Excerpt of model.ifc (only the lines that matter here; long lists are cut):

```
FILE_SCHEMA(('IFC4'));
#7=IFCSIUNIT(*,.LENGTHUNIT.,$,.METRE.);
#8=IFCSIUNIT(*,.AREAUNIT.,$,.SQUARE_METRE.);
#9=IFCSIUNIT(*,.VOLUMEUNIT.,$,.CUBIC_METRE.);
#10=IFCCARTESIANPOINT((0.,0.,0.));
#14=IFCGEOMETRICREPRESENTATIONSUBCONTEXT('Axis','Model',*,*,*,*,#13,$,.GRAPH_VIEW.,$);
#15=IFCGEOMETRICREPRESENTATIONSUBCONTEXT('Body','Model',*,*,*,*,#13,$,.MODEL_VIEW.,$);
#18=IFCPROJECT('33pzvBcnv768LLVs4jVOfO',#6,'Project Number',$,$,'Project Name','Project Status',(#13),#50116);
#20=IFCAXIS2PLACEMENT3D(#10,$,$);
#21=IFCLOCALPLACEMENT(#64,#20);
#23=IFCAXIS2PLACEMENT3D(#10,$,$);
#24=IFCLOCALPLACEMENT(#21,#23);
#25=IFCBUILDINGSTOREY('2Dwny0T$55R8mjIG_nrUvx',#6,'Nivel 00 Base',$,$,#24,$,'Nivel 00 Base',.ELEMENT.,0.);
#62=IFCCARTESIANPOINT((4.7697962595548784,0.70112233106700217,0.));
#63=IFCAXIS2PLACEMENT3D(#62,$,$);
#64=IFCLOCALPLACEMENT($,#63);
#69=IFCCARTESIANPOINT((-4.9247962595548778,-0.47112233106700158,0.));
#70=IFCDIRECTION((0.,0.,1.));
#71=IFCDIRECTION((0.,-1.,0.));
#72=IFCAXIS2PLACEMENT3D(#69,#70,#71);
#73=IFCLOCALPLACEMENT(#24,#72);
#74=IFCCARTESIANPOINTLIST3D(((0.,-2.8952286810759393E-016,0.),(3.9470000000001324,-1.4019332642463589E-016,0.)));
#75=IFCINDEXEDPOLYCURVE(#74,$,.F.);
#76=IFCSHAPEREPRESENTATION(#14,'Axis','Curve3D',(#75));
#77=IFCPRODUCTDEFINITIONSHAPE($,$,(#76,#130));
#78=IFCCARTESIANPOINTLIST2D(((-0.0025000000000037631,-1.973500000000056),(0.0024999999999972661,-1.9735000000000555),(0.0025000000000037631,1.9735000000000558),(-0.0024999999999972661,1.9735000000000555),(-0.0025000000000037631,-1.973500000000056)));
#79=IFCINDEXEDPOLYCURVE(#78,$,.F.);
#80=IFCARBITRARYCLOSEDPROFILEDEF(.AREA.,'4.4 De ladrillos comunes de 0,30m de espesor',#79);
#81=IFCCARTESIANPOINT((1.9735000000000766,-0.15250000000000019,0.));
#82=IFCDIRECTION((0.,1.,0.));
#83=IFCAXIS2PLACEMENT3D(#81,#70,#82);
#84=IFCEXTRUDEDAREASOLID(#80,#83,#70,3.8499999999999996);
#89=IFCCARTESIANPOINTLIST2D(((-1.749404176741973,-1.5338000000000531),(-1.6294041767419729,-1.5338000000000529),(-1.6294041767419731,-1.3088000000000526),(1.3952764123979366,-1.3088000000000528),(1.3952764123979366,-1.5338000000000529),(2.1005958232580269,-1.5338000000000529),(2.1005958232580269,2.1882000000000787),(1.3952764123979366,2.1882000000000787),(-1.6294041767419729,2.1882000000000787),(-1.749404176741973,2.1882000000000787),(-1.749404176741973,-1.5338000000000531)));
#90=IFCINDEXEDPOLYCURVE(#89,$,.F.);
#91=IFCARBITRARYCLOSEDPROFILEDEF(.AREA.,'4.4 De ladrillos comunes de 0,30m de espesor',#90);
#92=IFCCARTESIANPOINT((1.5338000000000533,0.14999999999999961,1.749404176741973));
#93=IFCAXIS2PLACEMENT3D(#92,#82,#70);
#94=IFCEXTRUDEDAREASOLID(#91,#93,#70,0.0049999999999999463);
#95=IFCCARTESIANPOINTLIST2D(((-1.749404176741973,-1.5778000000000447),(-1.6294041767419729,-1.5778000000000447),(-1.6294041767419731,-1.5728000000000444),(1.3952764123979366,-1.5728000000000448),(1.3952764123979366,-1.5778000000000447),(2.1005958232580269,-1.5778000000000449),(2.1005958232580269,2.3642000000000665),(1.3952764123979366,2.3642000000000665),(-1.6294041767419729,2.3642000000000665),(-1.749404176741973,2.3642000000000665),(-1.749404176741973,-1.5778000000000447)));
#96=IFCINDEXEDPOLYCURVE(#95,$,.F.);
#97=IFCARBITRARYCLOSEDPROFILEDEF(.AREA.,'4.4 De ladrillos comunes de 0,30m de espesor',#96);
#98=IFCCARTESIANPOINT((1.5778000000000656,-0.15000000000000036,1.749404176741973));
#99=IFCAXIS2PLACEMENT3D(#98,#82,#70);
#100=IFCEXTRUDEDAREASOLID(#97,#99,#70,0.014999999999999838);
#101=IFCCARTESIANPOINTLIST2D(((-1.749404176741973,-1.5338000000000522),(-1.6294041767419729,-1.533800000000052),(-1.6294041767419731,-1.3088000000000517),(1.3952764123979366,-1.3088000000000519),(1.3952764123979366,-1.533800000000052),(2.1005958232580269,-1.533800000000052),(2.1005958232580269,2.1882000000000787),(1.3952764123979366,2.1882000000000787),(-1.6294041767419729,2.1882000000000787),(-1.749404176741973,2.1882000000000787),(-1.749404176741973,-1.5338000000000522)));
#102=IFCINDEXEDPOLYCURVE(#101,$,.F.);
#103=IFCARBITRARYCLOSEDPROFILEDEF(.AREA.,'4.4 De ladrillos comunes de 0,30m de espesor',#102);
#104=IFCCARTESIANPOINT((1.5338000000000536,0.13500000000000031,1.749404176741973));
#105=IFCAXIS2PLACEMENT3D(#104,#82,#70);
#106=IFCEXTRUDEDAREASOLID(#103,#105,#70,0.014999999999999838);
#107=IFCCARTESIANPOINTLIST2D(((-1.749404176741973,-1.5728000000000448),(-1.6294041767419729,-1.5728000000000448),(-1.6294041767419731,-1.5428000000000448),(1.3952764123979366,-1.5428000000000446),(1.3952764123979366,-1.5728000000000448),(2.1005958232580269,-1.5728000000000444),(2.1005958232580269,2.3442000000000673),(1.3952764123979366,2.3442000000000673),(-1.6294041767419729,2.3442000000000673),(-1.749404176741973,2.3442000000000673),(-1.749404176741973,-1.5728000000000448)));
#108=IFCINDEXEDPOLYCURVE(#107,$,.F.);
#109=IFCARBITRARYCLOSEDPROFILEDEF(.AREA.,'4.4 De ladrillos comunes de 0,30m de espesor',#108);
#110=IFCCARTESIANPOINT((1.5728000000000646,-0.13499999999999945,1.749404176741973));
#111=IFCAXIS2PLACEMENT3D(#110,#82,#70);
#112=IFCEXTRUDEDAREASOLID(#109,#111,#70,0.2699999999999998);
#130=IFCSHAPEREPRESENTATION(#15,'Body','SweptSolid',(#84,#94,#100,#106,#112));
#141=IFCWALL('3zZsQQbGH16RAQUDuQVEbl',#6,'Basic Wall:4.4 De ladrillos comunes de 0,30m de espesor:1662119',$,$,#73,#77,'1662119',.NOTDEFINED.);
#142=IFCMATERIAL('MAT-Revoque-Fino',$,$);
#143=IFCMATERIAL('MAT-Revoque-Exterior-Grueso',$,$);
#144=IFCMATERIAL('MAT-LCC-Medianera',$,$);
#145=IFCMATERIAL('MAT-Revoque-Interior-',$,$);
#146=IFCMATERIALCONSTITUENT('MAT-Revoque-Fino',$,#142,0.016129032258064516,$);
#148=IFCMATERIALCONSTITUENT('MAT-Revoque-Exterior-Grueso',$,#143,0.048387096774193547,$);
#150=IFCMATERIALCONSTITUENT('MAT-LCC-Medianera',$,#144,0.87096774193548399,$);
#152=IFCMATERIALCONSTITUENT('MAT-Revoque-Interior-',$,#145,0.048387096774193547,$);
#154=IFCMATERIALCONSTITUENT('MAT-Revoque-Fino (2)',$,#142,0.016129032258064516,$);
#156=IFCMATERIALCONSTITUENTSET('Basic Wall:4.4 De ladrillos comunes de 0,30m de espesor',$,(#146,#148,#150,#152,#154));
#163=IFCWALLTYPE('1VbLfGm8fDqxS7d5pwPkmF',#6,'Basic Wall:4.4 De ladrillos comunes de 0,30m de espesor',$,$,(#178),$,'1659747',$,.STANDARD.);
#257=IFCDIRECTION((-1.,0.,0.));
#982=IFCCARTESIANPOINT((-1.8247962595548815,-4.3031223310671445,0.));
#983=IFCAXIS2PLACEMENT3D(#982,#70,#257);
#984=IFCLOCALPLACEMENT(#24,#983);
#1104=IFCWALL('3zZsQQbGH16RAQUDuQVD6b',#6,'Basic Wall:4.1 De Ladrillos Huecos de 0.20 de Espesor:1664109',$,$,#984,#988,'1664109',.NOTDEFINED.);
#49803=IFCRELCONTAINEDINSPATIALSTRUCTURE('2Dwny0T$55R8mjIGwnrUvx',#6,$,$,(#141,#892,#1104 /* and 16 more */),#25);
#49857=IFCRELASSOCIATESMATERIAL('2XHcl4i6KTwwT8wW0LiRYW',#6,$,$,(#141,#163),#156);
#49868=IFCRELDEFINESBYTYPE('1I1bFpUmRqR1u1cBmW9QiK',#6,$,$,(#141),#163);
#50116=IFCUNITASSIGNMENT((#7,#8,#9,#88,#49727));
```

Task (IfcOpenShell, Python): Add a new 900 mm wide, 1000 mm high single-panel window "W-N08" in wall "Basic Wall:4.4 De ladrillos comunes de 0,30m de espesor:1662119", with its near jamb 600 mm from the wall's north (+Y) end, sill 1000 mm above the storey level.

```python
import numpy as np
import ifcopenshell
import ifcopenshell.api.feature
import ifcopenshell.api.geometry
import ifcopenshell.api.root
import ifcopenshell.api.spatial
import ifcopenshell.geom
import ifcopenshell.util.element
import ifcopenshell.util.placement
import ifcopenshell.util.representation
import ifcopenshell.util.shape
import ifcopenshell.util.unit

model = ifcopenshell.open("model.ifc")
unit_scale = ifcopenshell.util.unit.calculate_unit_scale(model)
settings = ifcopenshell.geom.settings()


def volume(element):
    """Net volume in cubic metres, openings subtracted."""
    shape = ifcopenshell.geom.create_shape(settings, element)
    return ifcopenshell.util.shape.get_volume(shape.geometry)


wall = model.by_guid("3zZsQQbGH16RAQUDuQVEbl")
storey = ifcopenshell.util.element.get_container(wall, ifc_class="IfcBuildingStorey")
context = ifcopenshell.util.representation.get_context(model, "Model", "Body", "MODEL_VIEW")
before = volume(wall)

width, height, from_end, sill = 0.9, 1, 0.6, 1  # metres

# The wall runs along its own X axis, and the end named is its -X end.
wall_shape = ifcopenshell.geom.create_shape(settings, wall)
x, y, z = ifcopenshell.util.shape.get_vertices(wall_shape.geometry).T
start = x.min() + from_end
face, thickness = float(y.min()), float(y.max() - y.min())
wall_matrix = ifcopenshell.util.placement.get_local_placement(wall.ObjectPlacement)
level = ifcopenshell.util.placement.get_local_placement(storey.ObjectPlacement)[2, 3]


def in_wall(x, y):
    """Placement at x, y metres in the wall's axes, at sill height."""
    matrix = wall_matrix.copy()
    matrix[:, 3] = wall_matrix @ np.array([x / unit_scale, y / unit_scale, 0.0, 1.0])
    matrix[2, 3] = level + sill / unit_scale
    return matrix


# Opening: a box that overshoots both wall faces by 50 mm.
opening = ifcopenshell.api.root.create_entity(model, ifc_class="IfcOpeningElement", predefined_type="OPENING")
box = ifcopenshell.api.geometry.add_wall_representation(
    model, context=context, length=width, height=height, thickness=thickness + 0.1
)
ifcopenshell.api.geometry.assign_representation(model, product=opening, representation=box)
ifcopenshell.api.geometry.edit_object_placement(model, product=opening, matrix=in_wall(start, face - 0.05), is_si=False)
ifcopenshell.api.feature.add_feature(model, feature=opening, element=wall)

window = ifcopenshell.api.root.create_entity(model, ifc_class="IfcWindow", name="W-N08", predefined_type="WINDOW")
window.OverallWidth, window.OverallHeight = width / unit_scale, height / unit_scale
window.PartitioningType = "SINGLE_PANEL"
body = ifcopenshell.api.geometry.add_window_representation(
    model,
    context=context,
    overall_width=window.OverallWidth,
    overall_height=window.OverallHeight,
    partition_type="SINGLE_PANEL",
)
ifcopenshell.api.geometry.assign_representation(model, product=window, representation=body)
ifcopenshell.api.spatial.assign_container(model, products=[window], relating_structure=storey)
ifcopenshell.api.feature.add_filling(model, opening=opening, element=window)

# Centre the window in the wall's thickness.
ifcopenshell.api.geometry.edit_object_placement(model, product=window, matrix=in_wall(start, face), is_si=False)
window_shape = ifcopenshell.geom.create_shape(settings, window)
depth = ifcopenshell.util.shape.get_vertices(window_shape.geometry)[:, 1]
offset = face + thickness / 2 - (depth.min() + depth.max()) / 2
ifcopenshell.api.geometry.edit_object_placement(model, product=window, matrix=in_wall(start, offset), is_si=False)

after = volume(wall)

print(f"wall volume {before:.3f} -> {after:.3f} m3")

model.write("model_v2.ifc")
```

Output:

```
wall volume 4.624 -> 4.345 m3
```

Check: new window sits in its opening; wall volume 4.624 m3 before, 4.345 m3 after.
